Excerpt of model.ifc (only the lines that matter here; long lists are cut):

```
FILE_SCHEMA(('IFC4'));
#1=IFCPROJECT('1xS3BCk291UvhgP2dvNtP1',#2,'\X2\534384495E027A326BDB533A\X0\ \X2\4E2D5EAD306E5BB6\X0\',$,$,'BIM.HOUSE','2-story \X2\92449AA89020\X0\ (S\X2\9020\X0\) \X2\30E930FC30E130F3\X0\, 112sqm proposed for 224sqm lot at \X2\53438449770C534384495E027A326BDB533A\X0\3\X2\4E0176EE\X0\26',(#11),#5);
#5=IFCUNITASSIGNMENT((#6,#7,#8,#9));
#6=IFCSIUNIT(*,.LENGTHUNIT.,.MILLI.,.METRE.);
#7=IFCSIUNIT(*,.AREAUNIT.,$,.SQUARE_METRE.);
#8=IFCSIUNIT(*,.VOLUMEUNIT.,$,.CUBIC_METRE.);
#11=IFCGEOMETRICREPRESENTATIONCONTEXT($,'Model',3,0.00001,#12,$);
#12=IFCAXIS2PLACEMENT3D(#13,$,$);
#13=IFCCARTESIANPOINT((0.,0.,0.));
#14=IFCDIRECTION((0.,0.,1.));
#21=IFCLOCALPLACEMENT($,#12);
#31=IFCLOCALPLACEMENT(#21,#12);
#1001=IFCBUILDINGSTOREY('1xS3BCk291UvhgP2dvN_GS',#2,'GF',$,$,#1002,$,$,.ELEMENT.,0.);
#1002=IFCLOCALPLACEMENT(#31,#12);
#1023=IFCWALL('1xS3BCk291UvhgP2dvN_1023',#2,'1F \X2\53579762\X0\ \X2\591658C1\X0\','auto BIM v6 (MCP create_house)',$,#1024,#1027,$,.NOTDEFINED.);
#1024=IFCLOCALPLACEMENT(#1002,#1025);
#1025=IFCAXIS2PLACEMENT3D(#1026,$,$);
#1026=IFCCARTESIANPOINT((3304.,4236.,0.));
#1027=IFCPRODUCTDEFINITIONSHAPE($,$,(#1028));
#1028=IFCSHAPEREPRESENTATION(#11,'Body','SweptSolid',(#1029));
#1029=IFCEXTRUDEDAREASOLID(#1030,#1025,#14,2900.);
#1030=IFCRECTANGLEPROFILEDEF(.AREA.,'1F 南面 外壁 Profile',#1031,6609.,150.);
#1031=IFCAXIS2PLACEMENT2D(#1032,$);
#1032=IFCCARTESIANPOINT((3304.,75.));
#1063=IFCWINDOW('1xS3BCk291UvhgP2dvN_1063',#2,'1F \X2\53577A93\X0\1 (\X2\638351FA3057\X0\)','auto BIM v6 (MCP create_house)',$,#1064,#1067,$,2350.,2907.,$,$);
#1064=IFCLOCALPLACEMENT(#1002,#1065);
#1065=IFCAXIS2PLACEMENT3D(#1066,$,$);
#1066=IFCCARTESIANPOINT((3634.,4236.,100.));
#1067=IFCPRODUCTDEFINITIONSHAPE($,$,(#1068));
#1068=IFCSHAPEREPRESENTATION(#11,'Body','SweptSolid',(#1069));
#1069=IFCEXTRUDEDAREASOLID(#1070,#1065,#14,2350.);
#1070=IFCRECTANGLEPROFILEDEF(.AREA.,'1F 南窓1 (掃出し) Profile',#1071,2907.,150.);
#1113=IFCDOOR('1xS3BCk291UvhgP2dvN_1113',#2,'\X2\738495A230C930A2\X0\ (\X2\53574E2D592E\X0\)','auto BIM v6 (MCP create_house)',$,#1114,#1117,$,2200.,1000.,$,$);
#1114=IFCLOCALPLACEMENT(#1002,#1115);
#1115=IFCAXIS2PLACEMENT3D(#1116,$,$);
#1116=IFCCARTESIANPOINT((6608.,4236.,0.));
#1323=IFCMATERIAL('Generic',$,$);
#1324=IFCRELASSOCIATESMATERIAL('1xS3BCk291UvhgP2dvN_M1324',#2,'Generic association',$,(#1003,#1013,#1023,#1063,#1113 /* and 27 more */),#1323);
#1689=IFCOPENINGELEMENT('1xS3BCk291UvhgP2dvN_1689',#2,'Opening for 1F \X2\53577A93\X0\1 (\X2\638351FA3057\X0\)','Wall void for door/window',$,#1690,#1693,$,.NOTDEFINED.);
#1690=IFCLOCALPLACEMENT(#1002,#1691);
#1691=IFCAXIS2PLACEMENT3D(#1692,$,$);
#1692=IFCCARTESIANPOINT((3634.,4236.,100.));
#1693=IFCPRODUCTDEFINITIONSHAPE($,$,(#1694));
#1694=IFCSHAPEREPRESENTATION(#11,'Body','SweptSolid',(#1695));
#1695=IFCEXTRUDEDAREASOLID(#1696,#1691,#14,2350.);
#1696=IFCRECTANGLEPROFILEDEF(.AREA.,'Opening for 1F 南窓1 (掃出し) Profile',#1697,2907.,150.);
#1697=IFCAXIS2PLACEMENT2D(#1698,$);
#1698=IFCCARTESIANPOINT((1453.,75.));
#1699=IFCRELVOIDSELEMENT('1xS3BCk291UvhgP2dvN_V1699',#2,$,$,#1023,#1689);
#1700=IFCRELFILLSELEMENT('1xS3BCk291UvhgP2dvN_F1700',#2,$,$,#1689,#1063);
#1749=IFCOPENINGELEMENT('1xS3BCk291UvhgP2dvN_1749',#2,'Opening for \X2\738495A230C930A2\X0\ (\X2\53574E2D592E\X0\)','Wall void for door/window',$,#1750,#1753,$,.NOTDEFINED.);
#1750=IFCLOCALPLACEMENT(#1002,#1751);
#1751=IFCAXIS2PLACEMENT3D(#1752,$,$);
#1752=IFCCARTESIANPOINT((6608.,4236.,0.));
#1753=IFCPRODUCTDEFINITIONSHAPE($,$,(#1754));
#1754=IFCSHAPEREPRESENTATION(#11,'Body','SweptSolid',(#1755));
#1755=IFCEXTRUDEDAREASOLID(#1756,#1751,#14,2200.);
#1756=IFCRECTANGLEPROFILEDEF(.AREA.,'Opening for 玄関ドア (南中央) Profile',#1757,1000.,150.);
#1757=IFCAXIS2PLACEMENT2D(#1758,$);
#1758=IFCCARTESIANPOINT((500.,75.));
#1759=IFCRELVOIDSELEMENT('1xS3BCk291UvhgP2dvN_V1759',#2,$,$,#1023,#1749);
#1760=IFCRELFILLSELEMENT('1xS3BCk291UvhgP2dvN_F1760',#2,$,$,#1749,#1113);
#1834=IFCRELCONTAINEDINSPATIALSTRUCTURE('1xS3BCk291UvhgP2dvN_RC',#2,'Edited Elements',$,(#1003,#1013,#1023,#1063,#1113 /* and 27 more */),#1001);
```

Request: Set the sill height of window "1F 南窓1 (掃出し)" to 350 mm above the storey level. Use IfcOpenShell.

```python
import numpy as np
import ifcopenshell
import ifcopenshell.api.geometry
import ifcopenshell.geom
import ifcopenshell.util.element
import ifcopenshell.util.placement
import ifcopenshell.util.shape
import ifcopenshell.util.unit

model = ifcopenshell.open("model.ifc")
unit_scale = ifcopenshell.util.unit.calculate_unit_scale(model)

window = model.by_id(1063)
opening = window.FillsVoids[0].RelatingOpeningElement
storey = ifcopenshell.util.element.get_container(window, ifc_class="IfcBuildingStorey")
level = ifcopenshell.util.placement.get_local_placement(storey.ObjectPlacement)[2, 3]

# The opening's origin need not be at the sill, so measure its lowest point.
shape = ifcopenshell.geom.create_shape(ifcopenshell.geom.settings(), opening)
bottom = ifcopenshell.util.shape.get_shape_bottom_elevation(shape, shape.geometry) / unit_scale
dz = level + 0.35 / unit_scale - bottom

shift = np.array([0.0, 0.0, dz])
# The window is not placed relative to its opening, so move both.
for product in (opening, window):
    matrix = ifcopenshell.util.placement.get_local_placement(product.ObjectPlacement)
    matrix[:3, 3] += shift
    ifcopenshell.api.geometry.edit_object_placement(model, product=product, matrix=matrix, is_si=False)

print(f"moved by {dz * unit_scale:+.3f} m")

model.write("model_updated.ifc")
```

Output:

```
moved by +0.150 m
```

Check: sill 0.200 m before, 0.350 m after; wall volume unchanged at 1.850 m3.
